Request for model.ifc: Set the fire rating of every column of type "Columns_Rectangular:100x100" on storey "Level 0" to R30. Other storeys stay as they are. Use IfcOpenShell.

First a look at what the model holds.

```python
import ifcopenshell
import ifcopenshell.util.element

model = ifcopenshell.open("model.ifc")
print(model.schema)
storey = next(s for s in model.by_type("IfcBuildingStorey") if s.Name == "Level 0")
columns = [e for e in ifcopenshell.util.element.get_decomposition(storey) if e.is_a("IfcColumn")]
seen = {}
for e in columns:
    element_type = ifcopenshell.util.element.get_type(e)
    key = (element_type.Name if element_type != e and element_type else None, ifcopenshell.util.element.get_pset(e, "Pset_ColumnCommon", "FireRating"))
    seen[key] = seen.get(key, 0) + 1
for (name, value), count in sorted(seen.items(), key=str):
    print(count, "x", name, "|", value)
```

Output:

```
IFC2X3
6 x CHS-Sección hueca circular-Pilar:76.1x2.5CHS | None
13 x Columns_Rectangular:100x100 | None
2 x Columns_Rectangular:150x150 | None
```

```python
import ifcopenshell
import ifcopenshell.api.pset
import ifcopenshell.util.element

model = ifcopenshell.open("model.ifc")

storey = next(s for s in model.by_type("IfcBuildingStorey") if s.Name == "Level 0")
columns = [e for e in ifcopenshell.util.element.get_decomposition(storey) if e.is_a("IfcColumn")]

count = 0
for e in columns:
    element_type = ifcopenshell.util.element.get_type(e)
    if element_type in (None, e) or element_type.Name != "Columns_Rectangular:100x100":
        continue
    # add_pset returns the element's existing set when there is one.
    pset = ifcopenshell.api.pset.add_pset(model, product=e, name="Pset_ColumnCommon")
    ifcopenshell.api.pset.edit_pset(model, pset=pset, properties={"FireRating": "R30"})
    count += 1

print(count, "columns updated")

model.write("model_v2.ifc")
```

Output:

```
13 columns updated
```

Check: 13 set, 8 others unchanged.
